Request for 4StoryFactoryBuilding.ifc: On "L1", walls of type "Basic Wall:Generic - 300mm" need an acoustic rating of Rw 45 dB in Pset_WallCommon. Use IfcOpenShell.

First a look at what the model holds.

```python
import ifcopenshell
import ifcopenshell.util.element

model = ifcopenshell.open("4StoryFactoryBuilding.ifc")
print(model.schema)
storey = next(s for s in model.by_type("IfcBuildingStorey") if s.Name == "L1")
walls = [e for e in ifcopenshell.util.element.get_decomposition(storey) if e.is_a("IfcWall")]
seen = {}
for e in walls:
    element_type = ifcopenshell.util.element.get_type(e)
    key = (element_type.Name if element_type != e and element_type else None, ifcopenshell.util.element.get_pset(e, "Pset_WallCommon", "AcousticRating"))
    seen[key] = seen.get(key, 0) + 1
for (name, value), count in sorted(seen.items(), key=str):
    print(count, "x", name, "|", value)
```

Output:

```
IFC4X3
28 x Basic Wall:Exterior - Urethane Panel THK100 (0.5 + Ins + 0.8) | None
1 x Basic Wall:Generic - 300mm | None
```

```python
import ifcopenshell
import ifcopenshell.api.pset
import ifcopenshell.util.element

model = ifcopenshell.open("4StoryFactoryBuilding.ifc")

storey = next(s for s in model.by_type("IfcBuildingStorey") if s.Name == "L1")
walls = [e for e in ifcopenshell.util.element.get_decomposition(storey) if e.is_a("IfcWall")]

count = 0
for e in walls:
    element_type = ifcopenshell.util.element.get_type(e)
    if element_type in (None, e) or element_type.Name != "Basic Wall:Generic - 300mm":
        continue
    # add_pset returns the element's existing set when there is one.
    pset = ifcopenshell.api.pset.add_pset(model, product=e, name="Pset_WallCommon")
    ifcopenshell.api.pset.edit_pset(model, pset=pset, properties={"AcousticRating": "Rw 45 dB"})
    count += 1

print(count, "walls updated")

model.write("4StoryFactoryBuilding_v2.ifc")
```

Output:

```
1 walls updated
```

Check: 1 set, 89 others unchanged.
